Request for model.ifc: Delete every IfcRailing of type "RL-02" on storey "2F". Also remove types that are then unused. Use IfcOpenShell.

First a look at what the model holds.

```python
import ifcopenshell
import ifcopenshell.util.element

model = ifcopenshell.open("model.ifc")
print(model.schema)
storey = next(s for s in model.by_type("IfcBuildingStorey") if s.Name == "2F")
railings = [e for e in ifcopenshell.util.element.get_decomposition(storey) if e.is_a("IfcRailing")]
seen = {}
for e in railings:
    element_type = ifcopenshell.util.element.get_type(e)
    name = element_type.Name if element_type not in (None, e) else None
    seen[name] = seen.get(name, 0) + 1
for name, count in sorted(seen.items(), key=str):
    print(count, "x", name)
```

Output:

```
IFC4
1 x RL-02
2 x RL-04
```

```python
import ifcopenshell
import ifcopenshell.api.root
import ifcopenshell.util.element

model = ifcopenshell.open("model.ifc")

storey = next(s for s in model.by_type("IfcBuildingStorey") if s.Name == "2F")
railings = [e for e in ifcopenshell.util.element.get_decomposition(storey) if e.is_a("IfcRailing")]
targets = [e for e in railings if (t := ifcopenshell.util.element.get_type(e)) not in (None, e) and t.Name == "RL-02"]
types = {ifcopenshell.util.element.get_type(e) for e in targets} - {None, *targets}

for e in targets:
    ifcopenshell.api.root.remove_product(model, product=e)
print(len(targets), "removed")

unused = [t for t in types if not ifcopenshell.util.element.get_types(t)]
for t in unused:
    ifcopenshell.api.root.remove_product(model, product=t)
print(len(unused), "unused types removed")

model.write("model_rev.ifc")
```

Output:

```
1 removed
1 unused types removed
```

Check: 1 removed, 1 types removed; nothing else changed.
